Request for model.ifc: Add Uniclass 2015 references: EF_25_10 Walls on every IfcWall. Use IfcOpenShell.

First a look at what the model holds.

```python
import ifcopenshell

model = ifcopenshell.open("model.ifc")
print(model.schema)
print("classifications:", [c.Name for c in model.by_type("IfcClassification")])
for ifc_class in ("IfcDoor", "IfcRoof", "IfcStair", "IfcWall", "IfcWindow"):
    print(ifc_class, len(model.by_type(ifc_class)))
```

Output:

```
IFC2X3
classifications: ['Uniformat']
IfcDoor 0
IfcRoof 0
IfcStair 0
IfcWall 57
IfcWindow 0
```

```python
import ifcopenshell
import ifcopenshell.api.classification

model = ifcopenshell.open("model.ifc")

# IFC2X3 requires Source and Edition and has no link from the project to the system.
system = model.create_entity("IfcClassification", Source="NBS", Edition="2015", Name="Uniclass 2015")

codes = {
    "IfcWall": ("EF_25_10", "Walls"),
}
for ifc_class, (code, name) in codes.items():
    products = model.by_type(ifc_class)
    ifcopenshell.api.classification.add_reference(
        model, products=products, classification=system, identification=code, name=name
    )
    print(code, len(products))

model.write("model_updated.ifc")
```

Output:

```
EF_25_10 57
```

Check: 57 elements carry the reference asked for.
